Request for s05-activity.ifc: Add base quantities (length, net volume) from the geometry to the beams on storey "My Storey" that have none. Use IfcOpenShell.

First a look at what the model holds.

```python
import ifcopenshell
import ifcopenshell.util.element
import ifcopenshell.util.unit

model = ifcopenshell.open("s05-activity.ifc")
print(model.schema)
for unit_type in ("LENGTHUNIT", "AREAUNIT", "VOLUMEUNIT"):
    print(unit_type, ifcopenshell.util.unit.calculate_unit_scale(model, unit_type))
storey = next(s for s in model.by_type("IfcBuildingStorey") if s.Name == "My Storey")
beams = [e for e in ifcopenshell.util.element.get_decomposition(storey) if e.is_a("IfcBeam")]
for e in sorted(beams, key=lambda e: e.id()):
    print(e.id(), e.is_a(), e.Name, list(ifcopenshell.util.element.get_psets(e, qtos_only=True)), sep=" | ")
```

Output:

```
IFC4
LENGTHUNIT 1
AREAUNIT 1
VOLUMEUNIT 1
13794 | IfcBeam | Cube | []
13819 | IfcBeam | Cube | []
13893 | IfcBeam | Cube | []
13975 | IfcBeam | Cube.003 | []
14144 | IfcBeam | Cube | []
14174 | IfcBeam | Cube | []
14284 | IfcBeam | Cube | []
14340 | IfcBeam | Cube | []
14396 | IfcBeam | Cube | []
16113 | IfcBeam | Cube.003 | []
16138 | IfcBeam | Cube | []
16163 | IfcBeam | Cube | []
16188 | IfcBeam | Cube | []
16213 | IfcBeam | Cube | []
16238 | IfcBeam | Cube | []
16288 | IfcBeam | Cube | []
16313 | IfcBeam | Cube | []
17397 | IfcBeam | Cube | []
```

```python
import ifcopenshell
import ifcopenshell.api.pset
import ifcopenshell.geom
import ifcopenshell.util.element
import ifcopenshell.util.shape
import ifcopenshell.util.unit

model = ifcopenshell.open("s05-activity.ifc")
unit_scale = ifcopenshell.util.unit.calculate_unit_scale(model)
volume_scale = ifcopenshell.util.unit.calculate_unit_scale(model, "VOLUMEUNIT")
settings = ifcopenshell.geom.settings()

storey = next(s for s in model.by_type("IfcBuildingStorey") if s.Name == "My Storey")
beams = [e for e in ifcopenshell.util.element.get_decomposition(storey) if e.is_a("IfcBeam")]

for e in sorted(beams, key=lambda e: e.id()):
    if ifcopenshell.util.element.get_psets(e, qtos_only=True, should_inherit=False):
        continue
    # Geometry comes back in metres, in the element's own axes.
    shape = ifcopenshell.geom.create_shape(settings, e)
    values = {
        "Length": ifcopenshell.util.shape.get_max_xyz(shape.geometry) / unit_scale,
        "NetVolume": ifcopenshell.util.shape.get_volume(shape.geometry) / volume_scale,
    }
    qto = ifcopenshell.api.pset.add_qto(model, product=e, name="Qto_BeamBaseQuantities")
    ifcopenshell.api.pset.edit_qto(model, qto=qto, properties=values)
    print(e.id(), {k: round(v, 3) for k, v in values.items()})

model.write("s05-activity_edited.ifc")
```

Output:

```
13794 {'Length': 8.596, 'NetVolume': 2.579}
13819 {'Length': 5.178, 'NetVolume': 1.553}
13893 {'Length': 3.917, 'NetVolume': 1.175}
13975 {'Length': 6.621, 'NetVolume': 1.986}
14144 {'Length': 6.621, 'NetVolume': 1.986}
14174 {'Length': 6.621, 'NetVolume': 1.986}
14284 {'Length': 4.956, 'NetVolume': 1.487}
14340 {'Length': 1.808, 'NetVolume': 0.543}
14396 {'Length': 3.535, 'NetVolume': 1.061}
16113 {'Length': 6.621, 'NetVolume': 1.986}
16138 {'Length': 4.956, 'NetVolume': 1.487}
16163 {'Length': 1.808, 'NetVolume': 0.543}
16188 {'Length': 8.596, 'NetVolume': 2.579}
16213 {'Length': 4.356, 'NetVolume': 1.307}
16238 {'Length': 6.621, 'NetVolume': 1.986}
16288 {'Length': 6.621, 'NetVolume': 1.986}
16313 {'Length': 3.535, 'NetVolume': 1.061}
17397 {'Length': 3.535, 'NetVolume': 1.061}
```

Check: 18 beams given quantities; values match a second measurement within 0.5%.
